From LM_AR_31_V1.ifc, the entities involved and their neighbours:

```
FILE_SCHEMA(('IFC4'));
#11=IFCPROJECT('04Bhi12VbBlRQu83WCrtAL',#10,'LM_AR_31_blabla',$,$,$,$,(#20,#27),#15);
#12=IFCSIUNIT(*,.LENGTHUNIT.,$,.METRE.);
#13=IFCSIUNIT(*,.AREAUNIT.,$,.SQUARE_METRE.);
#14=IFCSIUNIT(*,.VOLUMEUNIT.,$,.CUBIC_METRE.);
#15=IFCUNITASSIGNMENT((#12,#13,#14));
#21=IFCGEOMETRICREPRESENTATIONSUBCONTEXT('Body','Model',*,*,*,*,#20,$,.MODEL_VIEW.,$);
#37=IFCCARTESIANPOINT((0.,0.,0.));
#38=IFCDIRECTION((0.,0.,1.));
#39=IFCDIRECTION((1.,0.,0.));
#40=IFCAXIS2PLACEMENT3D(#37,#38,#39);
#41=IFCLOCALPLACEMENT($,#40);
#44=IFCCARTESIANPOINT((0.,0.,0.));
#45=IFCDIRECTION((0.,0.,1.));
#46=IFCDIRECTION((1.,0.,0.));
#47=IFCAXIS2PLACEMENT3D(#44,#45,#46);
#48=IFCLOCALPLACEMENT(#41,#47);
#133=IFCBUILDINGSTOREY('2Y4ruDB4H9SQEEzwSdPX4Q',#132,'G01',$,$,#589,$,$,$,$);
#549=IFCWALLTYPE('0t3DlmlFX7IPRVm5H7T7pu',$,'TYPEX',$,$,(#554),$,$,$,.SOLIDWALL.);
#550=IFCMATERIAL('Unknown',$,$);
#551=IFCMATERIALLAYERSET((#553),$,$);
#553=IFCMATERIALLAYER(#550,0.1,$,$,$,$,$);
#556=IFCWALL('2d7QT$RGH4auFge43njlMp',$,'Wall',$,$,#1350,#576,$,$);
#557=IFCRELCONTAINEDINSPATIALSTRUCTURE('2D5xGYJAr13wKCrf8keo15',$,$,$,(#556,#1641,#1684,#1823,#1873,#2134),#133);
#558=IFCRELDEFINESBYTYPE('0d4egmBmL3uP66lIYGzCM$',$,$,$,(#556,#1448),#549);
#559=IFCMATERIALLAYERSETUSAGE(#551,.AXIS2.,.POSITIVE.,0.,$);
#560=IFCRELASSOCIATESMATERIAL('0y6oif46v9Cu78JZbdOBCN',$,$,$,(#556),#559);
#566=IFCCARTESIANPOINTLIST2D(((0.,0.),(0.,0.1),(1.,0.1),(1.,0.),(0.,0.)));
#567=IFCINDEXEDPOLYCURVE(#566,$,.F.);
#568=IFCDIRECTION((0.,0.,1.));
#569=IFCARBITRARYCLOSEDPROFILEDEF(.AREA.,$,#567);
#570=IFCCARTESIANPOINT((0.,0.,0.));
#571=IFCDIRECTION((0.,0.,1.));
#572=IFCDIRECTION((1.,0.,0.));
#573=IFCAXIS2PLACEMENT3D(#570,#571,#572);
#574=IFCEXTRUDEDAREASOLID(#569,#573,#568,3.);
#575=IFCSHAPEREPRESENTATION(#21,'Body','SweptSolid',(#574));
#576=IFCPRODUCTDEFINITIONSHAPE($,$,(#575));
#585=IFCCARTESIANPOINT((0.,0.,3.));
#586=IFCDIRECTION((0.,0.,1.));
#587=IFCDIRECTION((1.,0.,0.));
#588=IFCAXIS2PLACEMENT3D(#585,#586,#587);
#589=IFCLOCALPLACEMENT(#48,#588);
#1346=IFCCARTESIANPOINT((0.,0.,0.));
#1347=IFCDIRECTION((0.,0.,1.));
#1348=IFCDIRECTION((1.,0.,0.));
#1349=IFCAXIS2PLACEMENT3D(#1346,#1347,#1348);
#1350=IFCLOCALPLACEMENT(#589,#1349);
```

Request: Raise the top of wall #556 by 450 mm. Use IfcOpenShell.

```python
import ifcopenshell
import ifcopenshell.geom
import ifcopenshell.util.representation
import ifcopenshell.util.shape

model = ifcopenshell.open("LM_AR_31_V1.ifc")
settings = ifcopenshell.geom.settings()


def volume(element):
    """Net volume in cubic metres, openings subtracted."""
    shape = ifcopenshell.geom.create_shape(settings, element)
    return ifcopenshell.util.shape.get_volume(shape.geometry)


wall = model.by_guid("2d7QT$RGH4auFge43njlMp")
before = volume(wall)

body = ifcopenshell.util.representation.get_representation(wall, "Model", "Body")
solid = body.Items[0]
old_height = solid.Depth
solid.Depth += 0.45
after = volume(wall)

print(f"height {old_height:g} -> {solid.Depth:g}, volume {before:.3f} -> {after:.3f} m3")

model.write("LM_AR_31_V1_edited.ifc")
```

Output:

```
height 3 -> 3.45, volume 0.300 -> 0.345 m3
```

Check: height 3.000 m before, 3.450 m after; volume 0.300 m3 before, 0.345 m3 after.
